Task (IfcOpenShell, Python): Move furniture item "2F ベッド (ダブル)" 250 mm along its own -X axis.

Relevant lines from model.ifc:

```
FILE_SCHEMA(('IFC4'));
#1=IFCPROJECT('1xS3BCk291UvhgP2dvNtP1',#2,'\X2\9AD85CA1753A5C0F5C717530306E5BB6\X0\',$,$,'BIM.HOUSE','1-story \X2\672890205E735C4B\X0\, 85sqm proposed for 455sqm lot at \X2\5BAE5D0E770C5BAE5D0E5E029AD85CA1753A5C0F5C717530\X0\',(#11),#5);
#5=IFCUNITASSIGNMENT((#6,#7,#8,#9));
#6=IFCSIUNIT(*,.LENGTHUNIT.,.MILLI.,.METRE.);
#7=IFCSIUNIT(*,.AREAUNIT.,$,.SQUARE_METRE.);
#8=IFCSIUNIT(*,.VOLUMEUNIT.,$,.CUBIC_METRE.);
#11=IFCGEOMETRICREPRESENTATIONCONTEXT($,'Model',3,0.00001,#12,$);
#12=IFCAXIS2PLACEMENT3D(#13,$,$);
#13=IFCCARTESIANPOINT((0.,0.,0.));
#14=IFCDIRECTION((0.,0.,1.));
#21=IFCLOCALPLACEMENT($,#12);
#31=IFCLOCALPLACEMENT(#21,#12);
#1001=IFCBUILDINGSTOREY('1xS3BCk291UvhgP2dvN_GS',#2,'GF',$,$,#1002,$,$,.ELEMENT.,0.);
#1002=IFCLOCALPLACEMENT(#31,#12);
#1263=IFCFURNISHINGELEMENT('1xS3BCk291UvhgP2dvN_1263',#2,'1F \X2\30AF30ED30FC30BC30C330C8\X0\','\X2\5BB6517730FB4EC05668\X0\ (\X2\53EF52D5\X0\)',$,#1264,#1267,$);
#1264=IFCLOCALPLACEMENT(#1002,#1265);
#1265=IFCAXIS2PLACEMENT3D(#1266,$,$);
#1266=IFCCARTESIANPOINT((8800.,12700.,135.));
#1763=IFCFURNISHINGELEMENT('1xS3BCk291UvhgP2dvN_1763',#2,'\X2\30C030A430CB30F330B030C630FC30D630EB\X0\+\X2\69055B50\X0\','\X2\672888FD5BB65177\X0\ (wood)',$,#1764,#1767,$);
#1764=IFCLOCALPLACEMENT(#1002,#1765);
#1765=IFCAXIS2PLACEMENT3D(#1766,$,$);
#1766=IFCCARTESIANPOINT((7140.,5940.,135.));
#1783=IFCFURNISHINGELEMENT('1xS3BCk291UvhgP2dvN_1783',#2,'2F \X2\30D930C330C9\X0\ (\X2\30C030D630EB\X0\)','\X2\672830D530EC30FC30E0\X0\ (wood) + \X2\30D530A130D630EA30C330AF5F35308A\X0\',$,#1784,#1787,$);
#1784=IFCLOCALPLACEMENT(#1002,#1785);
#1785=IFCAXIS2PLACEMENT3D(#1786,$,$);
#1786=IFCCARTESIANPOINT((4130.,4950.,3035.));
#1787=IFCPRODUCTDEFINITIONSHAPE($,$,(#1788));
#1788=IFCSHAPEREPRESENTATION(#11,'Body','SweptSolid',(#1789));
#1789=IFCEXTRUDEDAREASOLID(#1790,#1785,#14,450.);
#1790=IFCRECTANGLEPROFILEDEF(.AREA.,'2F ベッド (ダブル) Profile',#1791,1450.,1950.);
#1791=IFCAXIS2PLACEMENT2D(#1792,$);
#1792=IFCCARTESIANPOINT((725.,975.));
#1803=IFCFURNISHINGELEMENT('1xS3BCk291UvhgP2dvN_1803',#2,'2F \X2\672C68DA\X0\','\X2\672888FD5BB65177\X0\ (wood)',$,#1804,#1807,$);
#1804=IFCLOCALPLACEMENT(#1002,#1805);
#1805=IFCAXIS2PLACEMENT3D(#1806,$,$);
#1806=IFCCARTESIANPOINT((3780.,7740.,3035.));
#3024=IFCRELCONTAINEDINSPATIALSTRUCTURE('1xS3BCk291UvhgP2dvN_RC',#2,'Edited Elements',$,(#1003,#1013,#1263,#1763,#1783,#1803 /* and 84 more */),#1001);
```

```python
import ifcopenshell
import ifcopenshell.api.geometry
import ifcopenshell.util.placement
import ifcopenshell.util.unit

model = ifcopenshell.open("model.ifc")
unit_scale = ifcopenshell.util.unit.calculate_unit_scale(model)

item = model.by_guid("1xS3BCk291UvhgP2dvN_1783")
matrix = ifcopenshell.util.placement.get_local_placement(item.ObjectPlacement)
matrix[:3, 3] -= matrix[:3, 0] * 0.25 / unit_scale
ifcopenshell.api.geometry.edit_object_placement(model, product=item, matrix=matrix, is_si=False)

print(ifcopenshell.util.placement.get_local_placement(item.ObjectPlacement).round(3) + 0.0)

model.write("model_v2.ifc")
```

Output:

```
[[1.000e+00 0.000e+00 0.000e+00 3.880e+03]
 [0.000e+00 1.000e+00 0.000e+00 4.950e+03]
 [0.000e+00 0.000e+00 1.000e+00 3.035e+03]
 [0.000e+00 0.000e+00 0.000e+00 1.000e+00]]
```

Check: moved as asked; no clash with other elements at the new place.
